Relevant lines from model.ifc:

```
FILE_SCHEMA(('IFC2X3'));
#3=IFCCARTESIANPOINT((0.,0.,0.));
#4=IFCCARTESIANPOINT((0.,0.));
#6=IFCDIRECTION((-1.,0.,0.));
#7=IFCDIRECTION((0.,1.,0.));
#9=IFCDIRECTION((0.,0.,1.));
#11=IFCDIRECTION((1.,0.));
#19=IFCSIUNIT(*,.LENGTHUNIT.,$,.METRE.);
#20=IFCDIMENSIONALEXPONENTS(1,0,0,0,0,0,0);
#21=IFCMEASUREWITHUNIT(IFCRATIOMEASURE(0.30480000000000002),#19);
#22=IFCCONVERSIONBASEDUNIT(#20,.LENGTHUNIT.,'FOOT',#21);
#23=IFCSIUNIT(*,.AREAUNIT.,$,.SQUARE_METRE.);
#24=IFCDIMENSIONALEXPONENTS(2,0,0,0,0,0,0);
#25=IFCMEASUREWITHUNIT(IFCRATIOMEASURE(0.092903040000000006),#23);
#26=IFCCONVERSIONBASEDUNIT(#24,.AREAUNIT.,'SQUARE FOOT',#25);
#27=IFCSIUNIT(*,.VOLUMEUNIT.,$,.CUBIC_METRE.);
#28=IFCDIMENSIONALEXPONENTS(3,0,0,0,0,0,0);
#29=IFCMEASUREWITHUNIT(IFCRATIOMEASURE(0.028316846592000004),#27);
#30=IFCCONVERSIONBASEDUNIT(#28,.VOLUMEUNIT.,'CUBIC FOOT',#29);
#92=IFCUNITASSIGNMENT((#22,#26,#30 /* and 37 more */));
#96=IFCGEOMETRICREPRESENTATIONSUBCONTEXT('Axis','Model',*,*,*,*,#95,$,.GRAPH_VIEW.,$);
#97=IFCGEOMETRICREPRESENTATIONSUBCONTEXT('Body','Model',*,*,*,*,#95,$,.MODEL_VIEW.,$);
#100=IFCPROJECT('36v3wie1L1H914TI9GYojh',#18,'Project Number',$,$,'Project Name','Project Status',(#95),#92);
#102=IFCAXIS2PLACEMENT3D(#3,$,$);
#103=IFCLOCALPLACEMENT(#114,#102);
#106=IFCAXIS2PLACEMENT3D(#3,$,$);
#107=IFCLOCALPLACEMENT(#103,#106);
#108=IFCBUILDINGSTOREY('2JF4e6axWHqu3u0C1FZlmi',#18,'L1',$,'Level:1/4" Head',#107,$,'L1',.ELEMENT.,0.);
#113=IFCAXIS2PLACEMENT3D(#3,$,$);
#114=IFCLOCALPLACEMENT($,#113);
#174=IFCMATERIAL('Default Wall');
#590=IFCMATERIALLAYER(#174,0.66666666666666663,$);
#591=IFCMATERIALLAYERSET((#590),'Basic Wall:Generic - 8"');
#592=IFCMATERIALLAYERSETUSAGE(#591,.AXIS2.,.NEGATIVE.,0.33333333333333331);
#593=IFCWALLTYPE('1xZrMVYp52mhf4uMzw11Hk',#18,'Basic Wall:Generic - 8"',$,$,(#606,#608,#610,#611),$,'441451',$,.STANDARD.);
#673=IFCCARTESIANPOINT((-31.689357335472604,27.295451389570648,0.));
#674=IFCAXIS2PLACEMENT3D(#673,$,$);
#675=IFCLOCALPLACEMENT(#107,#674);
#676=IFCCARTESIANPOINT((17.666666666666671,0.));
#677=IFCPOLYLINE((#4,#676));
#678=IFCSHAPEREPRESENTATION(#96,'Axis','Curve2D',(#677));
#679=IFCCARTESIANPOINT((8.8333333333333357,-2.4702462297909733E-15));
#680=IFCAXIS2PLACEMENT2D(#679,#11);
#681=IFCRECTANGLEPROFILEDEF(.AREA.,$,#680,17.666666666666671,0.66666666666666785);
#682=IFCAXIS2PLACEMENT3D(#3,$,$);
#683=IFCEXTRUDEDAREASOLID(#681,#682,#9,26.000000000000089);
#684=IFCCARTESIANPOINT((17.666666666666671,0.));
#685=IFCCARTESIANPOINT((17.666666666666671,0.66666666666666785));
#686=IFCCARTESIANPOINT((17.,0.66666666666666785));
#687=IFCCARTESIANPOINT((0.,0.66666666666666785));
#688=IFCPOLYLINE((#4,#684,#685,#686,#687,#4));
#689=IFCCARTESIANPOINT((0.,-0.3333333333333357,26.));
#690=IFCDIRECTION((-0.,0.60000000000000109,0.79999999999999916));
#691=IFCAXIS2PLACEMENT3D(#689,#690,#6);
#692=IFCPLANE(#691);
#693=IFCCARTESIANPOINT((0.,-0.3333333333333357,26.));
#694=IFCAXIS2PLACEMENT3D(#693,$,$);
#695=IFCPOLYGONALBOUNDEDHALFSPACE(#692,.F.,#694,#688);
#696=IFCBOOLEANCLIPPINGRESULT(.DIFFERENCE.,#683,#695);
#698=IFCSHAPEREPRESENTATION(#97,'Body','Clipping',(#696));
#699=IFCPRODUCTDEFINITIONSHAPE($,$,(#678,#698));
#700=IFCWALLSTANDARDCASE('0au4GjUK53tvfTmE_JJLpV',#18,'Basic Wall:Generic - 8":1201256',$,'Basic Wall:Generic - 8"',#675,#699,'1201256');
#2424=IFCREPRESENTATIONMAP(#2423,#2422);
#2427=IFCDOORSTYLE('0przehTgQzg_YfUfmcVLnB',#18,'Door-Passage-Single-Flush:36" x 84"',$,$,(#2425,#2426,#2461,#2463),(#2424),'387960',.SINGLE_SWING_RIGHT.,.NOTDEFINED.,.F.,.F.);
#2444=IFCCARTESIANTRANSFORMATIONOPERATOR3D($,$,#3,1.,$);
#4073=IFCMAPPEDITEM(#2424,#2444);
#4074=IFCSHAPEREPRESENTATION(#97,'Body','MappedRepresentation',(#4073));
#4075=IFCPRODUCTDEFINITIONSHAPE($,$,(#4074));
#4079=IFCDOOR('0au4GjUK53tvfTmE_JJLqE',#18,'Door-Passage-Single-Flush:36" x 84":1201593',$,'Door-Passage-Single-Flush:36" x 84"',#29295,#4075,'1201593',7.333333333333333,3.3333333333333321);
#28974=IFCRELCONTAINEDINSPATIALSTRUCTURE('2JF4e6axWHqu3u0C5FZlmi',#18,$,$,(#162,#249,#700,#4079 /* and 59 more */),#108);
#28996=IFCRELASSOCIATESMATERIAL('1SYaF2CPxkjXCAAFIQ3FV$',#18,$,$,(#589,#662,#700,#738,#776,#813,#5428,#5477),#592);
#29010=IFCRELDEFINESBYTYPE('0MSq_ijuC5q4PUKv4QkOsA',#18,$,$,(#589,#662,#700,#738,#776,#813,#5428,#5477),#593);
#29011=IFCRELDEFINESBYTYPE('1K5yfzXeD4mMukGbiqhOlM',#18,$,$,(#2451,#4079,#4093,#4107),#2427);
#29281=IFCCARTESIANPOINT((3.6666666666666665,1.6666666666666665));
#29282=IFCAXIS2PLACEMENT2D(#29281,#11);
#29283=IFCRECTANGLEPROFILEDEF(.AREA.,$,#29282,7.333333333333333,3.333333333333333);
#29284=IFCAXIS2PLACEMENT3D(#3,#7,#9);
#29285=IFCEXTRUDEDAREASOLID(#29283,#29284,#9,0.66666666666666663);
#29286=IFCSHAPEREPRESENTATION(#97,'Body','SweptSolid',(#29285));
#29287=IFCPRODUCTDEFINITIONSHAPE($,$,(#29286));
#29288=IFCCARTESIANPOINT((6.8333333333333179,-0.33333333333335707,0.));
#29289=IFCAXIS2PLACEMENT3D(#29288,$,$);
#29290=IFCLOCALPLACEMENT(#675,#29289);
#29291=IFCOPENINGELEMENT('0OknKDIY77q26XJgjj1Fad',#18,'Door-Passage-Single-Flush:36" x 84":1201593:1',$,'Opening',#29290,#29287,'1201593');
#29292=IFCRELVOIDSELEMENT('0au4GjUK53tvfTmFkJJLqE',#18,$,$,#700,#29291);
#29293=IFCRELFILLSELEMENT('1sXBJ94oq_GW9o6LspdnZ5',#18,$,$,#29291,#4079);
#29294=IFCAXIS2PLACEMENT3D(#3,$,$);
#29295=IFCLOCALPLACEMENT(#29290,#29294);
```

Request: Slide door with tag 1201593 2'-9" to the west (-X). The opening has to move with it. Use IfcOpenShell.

```python
import ifcopenshell
import ifcopenshell.api.geometry
import ifcopenshell.util.placement
import ifcopenshell.util.unit

model = ifcopenshell.open("model.ifc")
unit_scale = ifcopenshell.util.unit.calculate_unit_scale(model)

door = model.by_guid("0au4GjUK53tvfTmE_JJLqE")
opening = door.FillsVoids[0].RelatingOpeningElement
wall = opening.VoidsElements[0].RelatingBuildingElement

wall_matrix = ifcopenshell.util.placement.get_local_placement(wall.ObjectPlacement)
shift = wall_matrix[:3, 0] * -33 * 0.0254 / unit_scale
before = ifcopenshell.util.placement.get_local_placement(door.ObjectPlacement)[:3, 3].copy()

# The door is placed relative to its opening, so it follows when the opening moves.
matrix = ifcopenshell.util.placement.get_local_placement(opening.ObjectPlacement)
matrix[:3, 3] += shift
ifcopenshell.api.geometry.edit_object_placement(
    model, product=opening, matrix=matrix, is_si=False, should_transform_children=True
)

after = ifcopenshell.util.placement.get_local_placement(door.ObjectPlacement)[:3, 3]
print("door moved by", (after - before).round(3) + 0.0)

model.write("model_rev.ifc")
```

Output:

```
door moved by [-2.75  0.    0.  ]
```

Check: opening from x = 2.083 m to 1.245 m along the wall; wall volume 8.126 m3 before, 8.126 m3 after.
